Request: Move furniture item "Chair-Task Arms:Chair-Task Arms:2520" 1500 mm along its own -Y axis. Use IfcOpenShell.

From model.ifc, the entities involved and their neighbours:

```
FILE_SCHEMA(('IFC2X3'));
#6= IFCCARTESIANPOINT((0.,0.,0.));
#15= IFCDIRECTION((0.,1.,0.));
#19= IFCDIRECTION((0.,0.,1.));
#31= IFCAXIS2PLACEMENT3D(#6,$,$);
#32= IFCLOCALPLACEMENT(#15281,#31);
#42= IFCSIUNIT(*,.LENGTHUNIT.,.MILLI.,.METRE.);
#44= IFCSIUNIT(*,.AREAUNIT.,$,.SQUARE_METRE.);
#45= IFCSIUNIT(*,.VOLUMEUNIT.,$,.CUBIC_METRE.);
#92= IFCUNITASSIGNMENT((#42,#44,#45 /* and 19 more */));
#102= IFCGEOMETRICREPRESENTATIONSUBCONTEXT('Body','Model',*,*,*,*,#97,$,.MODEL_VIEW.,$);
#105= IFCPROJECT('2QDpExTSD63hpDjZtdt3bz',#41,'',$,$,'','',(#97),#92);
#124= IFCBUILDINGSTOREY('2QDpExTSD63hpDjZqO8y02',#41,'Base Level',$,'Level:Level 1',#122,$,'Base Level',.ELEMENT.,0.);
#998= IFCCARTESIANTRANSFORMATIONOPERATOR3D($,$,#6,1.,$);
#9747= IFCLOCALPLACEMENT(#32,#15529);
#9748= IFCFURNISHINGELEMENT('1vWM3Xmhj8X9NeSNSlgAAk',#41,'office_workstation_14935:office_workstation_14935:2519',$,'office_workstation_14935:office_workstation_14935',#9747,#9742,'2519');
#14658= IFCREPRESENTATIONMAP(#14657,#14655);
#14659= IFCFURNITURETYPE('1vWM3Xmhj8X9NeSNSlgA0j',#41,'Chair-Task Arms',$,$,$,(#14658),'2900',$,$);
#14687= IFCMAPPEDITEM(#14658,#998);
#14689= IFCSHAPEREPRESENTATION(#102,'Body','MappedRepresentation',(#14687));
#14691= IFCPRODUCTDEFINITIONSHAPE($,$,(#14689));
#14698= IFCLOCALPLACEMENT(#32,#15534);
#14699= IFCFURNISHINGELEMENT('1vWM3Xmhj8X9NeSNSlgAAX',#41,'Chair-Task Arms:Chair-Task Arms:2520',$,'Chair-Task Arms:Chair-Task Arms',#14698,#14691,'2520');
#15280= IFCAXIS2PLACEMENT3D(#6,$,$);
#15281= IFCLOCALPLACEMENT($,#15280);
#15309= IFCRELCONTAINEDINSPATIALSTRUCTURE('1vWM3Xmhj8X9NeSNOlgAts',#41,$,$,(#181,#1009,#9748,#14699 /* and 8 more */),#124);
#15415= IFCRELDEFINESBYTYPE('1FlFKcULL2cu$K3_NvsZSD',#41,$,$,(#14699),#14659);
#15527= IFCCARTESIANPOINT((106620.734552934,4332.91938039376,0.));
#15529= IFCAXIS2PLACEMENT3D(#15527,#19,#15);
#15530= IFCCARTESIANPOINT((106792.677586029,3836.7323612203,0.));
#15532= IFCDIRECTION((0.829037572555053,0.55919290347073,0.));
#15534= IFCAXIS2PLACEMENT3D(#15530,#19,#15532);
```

```python
import ifcopenshell
import ifcopenshell.api.geometry
import ifcopenshell.util.placement
import ifcopenshell.util.unit

model = ifcopenshell.open("model.ifc")
unit_scale = ifcopenshell.util.unit.calculate_unit_scale(model)

item = model.by_guid("1vWM3Xmhj8X9NeSNSlgAAX")
matrix = ifcopenshell.util.placement.get_local_placement(item.ObjectPlacement)
matrix[:3, 3] -= matrix[:3, 1] * 1.5 / unit_scale
ifcopenshell.api.geometry.edit_object_placement(model, product=item, matrix=matrix, is_si=False)

print(ifcopenshell.util.placement.get_local_placement(item.ObjectPlacement).round(3) + 0.0)

model.write("model_updated.ifc")
```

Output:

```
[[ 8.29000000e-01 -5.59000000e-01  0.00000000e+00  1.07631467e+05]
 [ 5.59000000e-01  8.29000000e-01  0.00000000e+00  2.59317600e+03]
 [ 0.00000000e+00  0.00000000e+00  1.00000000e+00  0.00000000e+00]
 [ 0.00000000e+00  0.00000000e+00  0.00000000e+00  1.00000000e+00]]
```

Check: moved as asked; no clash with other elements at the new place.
